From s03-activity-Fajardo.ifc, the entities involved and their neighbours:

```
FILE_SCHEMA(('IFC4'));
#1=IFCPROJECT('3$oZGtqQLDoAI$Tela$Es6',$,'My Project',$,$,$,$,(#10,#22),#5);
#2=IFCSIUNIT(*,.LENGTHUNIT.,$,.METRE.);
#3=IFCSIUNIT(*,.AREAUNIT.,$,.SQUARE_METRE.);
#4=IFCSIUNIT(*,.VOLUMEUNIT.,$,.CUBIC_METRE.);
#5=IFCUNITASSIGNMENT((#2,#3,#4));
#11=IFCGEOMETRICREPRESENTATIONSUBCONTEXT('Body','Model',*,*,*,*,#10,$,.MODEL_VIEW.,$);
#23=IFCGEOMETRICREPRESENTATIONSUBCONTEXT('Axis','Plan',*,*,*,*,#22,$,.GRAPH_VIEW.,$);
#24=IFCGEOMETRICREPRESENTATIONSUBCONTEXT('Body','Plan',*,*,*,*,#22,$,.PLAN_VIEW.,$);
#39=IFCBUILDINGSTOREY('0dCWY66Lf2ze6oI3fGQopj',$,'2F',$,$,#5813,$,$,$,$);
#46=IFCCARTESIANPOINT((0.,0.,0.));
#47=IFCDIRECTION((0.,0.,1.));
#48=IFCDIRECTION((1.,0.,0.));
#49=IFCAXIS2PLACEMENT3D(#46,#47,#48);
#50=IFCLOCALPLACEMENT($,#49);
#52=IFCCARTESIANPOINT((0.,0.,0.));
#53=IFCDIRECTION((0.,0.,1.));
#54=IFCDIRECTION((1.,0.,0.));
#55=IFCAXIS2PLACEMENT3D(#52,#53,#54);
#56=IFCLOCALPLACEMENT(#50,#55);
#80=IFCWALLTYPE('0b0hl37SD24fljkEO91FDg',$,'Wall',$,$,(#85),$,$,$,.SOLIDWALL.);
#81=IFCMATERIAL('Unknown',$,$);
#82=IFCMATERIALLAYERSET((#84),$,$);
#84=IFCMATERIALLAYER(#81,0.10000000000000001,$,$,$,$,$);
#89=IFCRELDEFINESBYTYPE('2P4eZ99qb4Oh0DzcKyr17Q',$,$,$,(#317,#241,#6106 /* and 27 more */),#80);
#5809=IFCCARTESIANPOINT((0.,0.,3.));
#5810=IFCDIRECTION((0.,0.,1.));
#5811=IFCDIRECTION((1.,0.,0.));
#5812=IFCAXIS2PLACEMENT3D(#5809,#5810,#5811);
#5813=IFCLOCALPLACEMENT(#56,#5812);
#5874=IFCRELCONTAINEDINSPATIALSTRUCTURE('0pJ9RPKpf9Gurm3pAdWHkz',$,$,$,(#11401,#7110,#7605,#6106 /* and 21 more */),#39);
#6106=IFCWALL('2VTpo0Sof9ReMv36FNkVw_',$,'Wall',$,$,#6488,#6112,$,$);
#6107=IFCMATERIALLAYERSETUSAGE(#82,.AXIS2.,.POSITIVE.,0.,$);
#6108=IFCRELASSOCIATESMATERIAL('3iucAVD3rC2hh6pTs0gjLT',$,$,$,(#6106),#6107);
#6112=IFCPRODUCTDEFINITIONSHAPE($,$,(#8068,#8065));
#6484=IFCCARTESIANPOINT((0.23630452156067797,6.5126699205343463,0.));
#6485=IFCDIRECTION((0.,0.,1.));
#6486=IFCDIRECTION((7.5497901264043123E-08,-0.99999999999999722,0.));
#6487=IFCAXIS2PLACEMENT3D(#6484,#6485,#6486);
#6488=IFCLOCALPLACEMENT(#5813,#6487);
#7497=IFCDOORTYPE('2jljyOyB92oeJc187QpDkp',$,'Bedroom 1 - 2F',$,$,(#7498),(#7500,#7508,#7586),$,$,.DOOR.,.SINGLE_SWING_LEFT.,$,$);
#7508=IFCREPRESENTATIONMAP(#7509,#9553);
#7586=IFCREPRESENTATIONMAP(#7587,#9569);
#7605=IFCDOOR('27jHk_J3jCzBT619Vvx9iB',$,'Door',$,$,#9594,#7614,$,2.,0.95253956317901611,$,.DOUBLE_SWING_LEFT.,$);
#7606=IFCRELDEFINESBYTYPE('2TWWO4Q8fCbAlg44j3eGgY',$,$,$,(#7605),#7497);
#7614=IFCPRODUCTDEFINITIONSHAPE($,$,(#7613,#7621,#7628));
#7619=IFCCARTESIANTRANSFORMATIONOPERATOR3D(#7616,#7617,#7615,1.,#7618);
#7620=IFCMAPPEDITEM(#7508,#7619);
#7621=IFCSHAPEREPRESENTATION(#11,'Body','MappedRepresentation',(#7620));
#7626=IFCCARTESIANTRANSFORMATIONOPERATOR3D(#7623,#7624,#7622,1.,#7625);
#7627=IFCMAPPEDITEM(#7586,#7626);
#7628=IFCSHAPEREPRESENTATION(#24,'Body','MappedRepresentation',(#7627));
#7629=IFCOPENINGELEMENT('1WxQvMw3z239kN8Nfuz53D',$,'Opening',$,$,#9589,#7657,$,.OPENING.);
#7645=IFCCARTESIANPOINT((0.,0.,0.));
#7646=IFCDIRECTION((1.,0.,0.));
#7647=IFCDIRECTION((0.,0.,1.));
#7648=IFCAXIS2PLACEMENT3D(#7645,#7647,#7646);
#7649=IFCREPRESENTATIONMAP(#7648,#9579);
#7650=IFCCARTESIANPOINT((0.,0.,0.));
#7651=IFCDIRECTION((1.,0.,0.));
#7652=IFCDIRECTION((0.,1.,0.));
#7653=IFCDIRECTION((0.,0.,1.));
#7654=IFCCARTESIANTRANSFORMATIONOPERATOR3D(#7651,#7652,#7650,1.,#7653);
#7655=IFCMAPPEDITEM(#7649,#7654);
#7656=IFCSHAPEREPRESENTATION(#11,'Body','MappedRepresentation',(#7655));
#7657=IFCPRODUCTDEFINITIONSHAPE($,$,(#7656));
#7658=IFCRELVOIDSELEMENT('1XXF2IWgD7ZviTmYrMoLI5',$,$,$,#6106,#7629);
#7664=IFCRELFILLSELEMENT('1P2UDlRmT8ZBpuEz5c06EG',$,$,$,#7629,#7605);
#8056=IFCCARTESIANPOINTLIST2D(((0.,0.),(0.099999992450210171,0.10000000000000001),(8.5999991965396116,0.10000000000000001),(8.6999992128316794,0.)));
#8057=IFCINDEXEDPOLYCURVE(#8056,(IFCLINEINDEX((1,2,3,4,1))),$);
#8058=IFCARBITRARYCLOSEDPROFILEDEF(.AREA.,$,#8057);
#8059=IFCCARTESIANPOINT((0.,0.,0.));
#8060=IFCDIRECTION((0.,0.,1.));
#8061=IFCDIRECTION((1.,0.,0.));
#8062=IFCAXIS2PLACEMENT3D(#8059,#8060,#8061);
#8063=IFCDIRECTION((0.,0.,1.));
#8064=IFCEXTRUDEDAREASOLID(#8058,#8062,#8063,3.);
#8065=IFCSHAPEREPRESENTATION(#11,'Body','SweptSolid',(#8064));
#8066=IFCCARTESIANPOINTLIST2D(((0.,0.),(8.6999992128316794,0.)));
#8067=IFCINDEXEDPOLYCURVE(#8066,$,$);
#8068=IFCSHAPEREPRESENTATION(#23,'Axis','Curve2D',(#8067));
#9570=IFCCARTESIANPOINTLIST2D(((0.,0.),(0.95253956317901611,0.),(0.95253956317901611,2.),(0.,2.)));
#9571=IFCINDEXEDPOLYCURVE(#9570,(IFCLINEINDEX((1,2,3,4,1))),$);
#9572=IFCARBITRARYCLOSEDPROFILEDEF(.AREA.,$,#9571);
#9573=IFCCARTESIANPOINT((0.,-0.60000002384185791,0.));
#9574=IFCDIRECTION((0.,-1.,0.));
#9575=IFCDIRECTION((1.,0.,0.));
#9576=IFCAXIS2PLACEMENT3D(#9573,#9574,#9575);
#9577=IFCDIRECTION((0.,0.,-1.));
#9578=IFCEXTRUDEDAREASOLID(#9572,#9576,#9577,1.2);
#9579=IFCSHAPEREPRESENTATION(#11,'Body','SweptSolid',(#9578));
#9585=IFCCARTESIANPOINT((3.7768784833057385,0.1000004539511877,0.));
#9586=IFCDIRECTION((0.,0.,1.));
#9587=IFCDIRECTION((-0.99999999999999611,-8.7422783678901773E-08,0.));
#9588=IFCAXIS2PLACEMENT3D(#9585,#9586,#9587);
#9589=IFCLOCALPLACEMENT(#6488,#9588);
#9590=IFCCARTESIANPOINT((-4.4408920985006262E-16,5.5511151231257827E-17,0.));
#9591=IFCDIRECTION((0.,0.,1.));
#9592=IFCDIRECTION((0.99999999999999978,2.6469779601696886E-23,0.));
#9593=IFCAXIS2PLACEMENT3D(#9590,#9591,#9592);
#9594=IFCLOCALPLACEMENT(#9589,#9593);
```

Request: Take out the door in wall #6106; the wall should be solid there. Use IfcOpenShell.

```python
import ifcopenshell
import ifcopenshell.api.feature
import ifcopenshell.api.root
import ifcopenshell.geom
import ifcopenshell.util.shape

model = ifcopenshell.open("s03-activity-Fajardo.ifc")
settings = ifcopenshell.geom.settings()


def volume(element):
    """Net volume in cubic metres, openings subtracted."""
    shape = ifcopenshell.geom.create_shape(settings, element)
    return ifcopenshell.util.shape.get_volume(shape.geometry)


door = model.by_guid("27jHk_J3jCzBT619Vvx9iB")
opening = door.FillsVoids[0].RelatingOpeningElement
wall = opening.VoidsElements[0].RelatingBuildingElement
before = volume(wall)

ifcopenshell.api.root.remove_product(model, product=door)
ifcopenshell.api.feature.remove_feature(model, feature=opening)

after = volume(wall)

print(f"wall volume {before:.3f} -> {after:.3f} m3")

model.write("s03-activity-Fajardo_v2.ifc")
```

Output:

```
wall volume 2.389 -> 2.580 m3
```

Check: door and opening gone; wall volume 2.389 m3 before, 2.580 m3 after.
